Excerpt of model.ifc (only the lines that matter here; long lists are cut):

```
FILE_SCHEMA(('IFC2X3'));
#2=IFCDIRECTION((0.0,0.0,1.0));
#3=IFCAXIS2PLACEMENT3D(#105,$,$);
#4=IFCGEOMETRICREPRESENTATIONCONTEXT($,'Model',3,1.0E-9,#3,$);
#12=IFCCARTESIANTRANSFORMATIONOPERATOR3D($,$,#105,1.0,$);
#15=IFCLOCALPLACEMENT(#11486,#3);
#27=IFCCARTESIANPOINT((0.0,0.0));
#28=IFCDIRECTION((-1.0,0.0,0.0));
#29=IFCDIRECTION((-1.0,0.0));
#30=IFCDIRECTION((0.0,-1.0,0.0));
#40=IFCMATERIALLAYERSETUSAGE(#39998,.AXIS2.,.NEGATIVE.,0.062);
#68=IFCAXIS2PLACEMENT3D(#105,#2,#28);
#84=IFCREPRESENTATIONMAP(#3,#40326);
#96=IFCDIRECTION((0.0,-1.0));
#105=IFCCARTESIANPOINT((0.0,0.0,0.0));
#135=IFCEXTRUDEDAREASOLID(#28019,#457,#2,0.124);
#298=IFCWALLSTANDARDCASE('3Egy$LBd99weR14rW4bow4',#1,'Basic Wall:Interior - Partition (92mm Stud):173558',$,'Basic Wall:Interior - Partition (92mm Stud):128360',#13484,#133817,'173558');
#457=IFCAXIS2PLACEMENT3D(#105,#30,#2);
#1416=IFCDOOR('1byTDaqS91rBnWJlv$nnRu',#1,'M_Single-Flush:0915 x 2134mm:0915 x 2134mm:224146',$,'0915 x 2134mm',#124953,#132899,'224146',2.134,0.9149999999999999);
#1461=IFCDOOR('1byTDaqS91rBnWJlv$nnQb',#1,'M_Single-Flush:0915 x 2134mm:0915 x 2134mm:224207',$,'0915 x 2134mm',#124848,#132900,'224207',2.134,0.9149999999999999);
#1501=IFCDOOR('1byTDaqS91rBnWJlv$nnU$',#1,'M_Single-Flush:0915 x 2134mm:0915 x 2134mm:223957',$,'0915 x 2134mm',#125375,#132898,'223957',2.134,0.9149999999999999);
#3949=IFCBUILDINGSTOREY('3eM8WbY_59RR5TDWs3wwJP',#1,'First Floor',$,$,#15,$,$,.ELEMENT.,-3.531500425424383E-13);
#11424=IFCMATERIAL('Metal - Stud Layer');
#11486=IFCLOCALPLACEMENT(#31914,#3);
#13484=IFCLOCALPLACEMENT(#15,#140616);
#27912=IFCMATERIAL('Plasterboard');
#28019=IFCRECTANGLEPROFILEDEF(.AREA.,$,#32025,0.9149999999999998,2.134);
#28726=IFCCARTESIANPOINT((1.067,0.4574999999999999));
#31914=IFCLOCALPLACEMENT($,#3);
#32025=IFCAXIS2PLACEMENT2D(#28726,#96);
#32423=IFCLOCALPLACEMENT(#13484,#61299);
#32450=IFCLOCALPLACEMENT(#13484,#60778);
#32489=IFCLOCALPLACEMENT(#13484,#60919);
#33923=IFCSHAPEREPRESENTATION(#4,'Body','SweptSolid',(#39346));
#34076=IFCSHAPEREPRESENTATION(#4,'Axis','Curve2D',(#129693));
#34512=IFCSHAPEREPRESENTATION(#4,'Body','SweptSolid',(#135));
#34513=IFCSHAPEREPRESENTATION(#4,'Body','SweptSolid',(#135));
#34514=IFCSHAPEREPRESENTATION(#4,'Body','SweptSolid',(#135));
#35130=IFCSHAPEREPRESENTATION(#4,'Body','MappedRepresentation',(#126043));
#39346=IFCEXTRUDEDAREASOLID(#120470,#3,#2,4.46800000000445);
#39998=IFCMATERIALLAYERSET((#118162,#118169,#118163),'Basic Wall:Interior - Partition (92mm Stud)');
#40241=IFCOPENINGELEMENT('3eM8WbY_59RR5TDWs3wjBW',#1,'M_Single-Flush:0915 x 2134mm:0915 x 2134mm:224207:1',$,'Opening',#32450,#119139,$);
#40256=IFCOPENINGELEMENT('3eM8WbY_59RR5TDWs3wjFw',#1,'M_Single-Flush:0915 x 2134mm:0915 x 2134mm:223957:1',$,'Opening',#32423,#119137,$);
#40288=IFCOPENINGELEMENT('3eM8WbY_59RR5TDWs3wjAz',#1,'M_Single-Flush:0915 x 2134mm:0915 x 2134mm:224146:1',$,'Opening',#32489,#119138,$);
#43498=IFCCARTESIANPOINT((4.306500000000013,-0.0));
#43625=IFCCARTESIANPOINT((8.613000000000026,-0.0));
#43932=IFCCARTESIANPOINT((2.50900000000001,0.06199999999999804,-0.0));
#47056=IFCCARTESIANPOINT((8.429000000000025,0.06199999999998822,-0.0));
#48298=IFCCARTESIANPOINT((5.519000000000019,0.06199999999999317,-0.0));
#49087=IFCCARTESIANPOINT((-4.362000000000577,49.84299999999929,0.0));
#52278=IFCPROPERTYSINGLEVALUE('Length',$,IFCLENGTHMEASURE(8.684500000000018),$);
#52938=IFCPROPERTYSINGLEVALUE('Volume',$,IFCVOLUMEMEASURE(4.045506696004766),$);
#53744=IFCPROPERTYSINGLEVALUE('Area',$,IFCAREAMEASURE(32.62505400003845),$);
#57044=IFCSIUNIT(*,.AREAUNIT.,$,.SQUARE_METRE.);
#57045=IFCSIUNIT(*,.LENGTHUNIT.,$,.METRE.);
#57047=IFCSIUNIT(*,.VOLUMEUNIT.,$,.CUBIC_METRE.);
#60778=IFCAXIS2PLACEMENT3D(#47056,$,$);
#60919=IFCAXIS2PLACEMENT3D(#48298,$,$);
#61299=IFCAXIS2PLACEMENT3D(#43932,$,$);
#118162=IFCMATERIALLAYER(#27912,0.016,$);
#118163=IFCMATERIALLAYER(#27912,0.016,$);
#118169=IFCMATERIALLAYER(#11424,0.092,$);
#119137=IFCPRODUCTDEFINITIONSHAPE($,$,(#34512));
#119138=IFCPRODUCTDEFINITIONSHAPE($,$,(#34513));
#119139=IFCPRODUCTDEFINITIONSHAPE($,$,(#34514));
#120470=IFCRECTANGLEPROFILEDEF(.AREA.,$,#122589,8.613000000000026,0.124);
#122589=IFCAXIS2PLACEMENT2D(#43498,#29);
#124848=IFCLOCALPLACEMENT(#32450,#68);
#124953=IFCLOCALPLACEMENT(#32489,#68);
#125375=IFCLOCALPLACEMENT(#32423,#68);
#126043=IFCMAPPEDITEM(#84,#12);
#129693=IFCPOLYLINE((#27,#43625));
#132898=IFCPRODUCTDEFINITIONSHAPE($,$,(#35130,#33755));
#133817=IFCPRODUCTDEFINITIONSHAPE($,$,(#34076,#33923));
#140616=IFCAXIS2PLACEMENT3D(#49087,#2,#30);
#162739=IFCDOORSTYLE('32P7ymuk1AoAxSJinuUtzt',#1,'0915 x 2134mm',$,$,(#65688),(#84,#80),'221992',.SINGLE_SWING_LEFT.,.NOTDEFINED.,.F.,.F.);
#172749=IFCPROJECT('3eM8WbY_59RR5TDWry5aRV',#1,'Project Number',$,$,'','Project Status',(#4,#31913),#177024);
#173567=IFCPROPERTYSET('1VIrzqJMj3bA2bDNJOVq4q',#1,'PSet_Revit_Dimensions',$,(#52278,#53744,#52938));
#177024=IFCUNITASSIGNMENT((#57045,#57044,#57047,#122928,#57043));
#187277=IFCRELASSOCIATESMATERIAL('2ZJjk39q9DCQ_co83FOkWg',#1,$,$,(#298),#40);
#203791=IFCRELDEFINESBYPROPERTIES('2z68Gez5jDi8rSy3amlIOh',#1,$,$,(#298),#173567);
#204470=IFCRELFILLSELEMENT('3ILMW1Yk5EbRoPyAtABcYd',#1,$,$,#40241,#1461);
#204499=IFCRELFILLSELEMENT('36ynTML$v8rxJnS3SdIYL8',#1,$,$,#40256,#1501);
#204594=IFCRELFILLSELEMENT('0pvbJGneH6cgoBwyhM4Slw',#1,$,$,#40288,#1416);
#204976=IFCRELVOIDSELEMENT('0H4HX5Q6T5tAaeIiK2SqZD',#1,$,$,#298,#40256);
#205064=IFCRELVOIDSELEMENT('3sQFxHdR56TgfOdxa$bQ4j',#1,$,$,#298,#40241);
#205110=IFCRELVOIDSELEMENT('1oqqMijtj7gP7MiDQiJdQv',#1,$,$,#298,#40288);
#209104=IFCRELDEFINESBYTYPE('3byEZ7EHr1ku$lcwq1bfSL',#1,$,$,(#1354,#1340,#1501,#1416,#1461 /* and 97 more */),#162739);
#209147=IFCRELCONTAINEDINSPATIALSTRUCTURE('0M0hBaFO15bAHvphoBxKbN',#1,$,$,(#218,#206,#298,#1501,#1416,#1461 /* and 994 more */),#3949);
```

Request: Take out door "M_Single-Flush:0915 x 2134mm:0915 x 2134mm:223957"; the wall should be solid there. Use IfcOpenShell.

```python
import ifcopenshell
import ifcopenshell.api.feature
import ifcopenshell.api.pset
import ifcopenshell.api.root
import ifcopenshell.geom
import ifcopenshell.util.element
import ifcopenshell.util.shape
import ifcopenshell.util.unit

model = ifcopenshell.open("model.ifc")
area_scale = ifcopenshell.util.unit.calculate_unit_scale(model, "AREAUNIT")
volume_scale = ifcopenshell.util.unit.calculate_unit_scale(model, "VOLUMEUNIT")
settings = ifcopenshell.geom.settings()


def volume(element):
    """Net volume in cubic metres, openings subtracted."""
    shape = ifcopenshell.geom.create_shape(settings, element)
    return ifcopenshell.util.shape.get_volume(shape.geometry)


door = model.by_id(1501)
opening = door.FillsVoids[0].RelatingOpeningElement
wall = opening.VoidsElements[0].RelatingBuildingElement
before = volume(wall)

ifcopenshell.api.root.remove_product(model, product=door)
ifcopenshell.api.feature.remove_feature(model, feature=opening)

after = volume(wall)
thickness = 0.124  # wall thickness in metres

# Update the wall's stored quantities.
pset = model.by_id(ifcopenshell.util.element.get_pset(wall, "PSet_Revit_Dimensions", should_inherit=False)["id"])
ifcopenshell.api.pset.edit_pset(model, pset=pset, properties={
    "Area": model.create_entity("IfcAreaMeasure", after / thickness / area_scale),
    "Volume": model.create_entity("IfcVolumeMeasure", after / volume_scale),
})

print(f"wall volume {before:.3f} -> {after:.3f} m3")

model.write("model_edited.ifc")
```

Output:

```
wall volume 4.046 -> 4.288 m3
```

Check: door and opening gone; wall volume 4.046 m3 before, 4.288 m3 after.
